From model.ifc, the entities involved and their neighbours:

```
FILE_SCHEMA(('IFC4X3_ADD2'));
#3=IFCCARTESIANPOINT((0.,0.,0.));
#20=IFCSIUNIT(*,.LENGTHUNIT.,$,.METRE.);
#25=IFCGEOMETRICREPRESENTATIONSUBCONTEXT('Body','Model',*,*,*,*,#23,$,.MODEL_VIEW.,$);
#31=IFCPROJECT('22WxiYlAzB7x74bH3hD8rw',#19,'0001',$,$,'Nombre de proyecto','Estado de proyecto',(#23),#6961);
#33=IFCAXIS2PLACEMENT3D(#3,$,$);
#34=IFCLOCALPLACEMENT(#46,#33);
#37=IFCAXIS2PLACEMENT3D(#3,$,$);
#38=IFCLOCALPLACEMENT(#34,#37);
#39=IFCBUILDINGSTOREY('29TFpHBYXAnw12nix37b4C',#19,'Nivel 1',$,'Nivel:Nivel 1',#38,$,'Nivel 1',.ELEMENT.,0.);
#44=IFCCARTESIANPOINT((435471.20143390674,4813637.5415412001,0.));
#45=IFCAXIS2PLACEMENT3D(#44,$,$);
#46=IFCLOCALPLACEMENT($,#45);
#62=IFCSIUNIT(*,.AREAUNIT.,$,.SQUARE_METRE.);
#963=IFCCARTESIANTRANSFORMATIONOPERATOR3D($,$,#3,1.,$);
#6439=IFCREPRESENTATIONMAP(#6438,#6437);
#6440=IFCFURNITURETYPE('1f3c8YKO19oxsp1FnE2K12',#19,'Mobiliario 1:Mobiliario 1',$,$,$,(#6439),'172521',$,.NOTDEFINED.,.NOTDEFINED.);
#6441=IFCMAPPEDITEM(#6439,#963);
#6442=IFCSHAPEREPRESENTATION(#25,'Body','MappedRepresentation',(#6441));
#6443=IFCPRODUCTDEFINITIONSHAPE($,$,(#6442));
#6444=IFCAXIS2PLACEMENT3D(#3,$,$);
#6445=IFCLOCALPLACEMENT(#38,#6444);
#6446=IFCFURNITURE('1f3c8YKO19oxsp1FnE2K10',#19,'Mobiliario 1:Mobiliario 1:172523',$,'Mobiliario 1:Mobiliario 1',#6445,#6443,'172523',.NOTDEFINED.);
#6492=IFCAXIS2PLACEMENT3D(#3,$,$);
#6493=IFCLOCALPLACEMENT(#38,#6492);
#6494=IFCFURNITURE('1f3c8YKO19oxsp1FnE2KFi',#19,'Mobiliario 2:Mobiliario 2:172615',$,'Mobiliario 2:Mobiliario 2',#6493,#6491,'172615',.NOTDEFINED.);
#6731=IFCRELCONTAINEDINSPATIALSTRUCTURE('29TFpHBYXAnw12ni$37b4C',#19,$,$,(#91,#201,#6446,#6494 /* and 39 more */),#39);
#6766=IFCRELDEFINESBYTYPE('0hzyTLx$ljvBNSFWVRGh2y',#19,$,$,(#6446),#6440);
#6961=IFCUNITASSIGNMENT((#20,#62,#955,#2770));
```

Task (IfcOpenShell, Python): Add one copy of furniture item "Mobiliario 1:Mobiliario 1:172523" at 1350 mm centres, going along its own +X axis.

```python
import ifcopenshell
import ifcopenshell.api.geometry
import ifcopenshell.api.root
import ifcopenshell.util.element
import ifcopenshell.util.placement
import ifcopenshell.util.unit

model = ifcopenshell.open("model.ifc")
unit_scale = ifcopenshell.util.unit.calculate_unit_scale(model)


def reuse_history(source, copy):
    """copy_class also copies each property set's owner history, people and application; keep the originals."""
    for rel in copy.IsDefinedBy:
        if rel.is_a("IfcRelDefinesByProperties") and (history := rel.RelatingPropertyDefinition.OwnerHistory):
            rel.RelatingPropertyDefinition.OwnerHistory = source.OwnerHistory
            ifcopenshell.util.element.remove_deep2(model, history)


source = model.by_guid("1f3c8YKO19oxsp1FnE2K10")
base = ifcopenshell.util.placement.get_local_placement(source.ObjectPlacement)
step = base[:3, 0] * 1.35 / unit_scale

for i in range(1, 2):
    copy = ifcopenshell.api.root.copy_class(model, product=source)
    copy.Representation = ifcopenshell.util.element.copy_deep(
        model, source.Representation, exclude=["IfcGeometricRepresentationContext", "IfcRepresentationMap"]
    )
    copy.Name = "Mobiliario 1:Mobiliario 1"
    copy.Tag = None
    reuse_history(source, copy)
    matrix = base.copy()
    matrix[:3, 3] += i * step
    print("added at", matrix[:3, 3].round(3) + 0.0)
    ifcopenshell.api.geometry.edit_object_placement(model, product=copy, matrix=matrix, is_si=False)

model.write("model_updated.ifc")
```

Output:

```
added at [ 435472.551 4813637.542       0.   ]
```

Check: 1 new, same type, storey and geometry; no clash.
